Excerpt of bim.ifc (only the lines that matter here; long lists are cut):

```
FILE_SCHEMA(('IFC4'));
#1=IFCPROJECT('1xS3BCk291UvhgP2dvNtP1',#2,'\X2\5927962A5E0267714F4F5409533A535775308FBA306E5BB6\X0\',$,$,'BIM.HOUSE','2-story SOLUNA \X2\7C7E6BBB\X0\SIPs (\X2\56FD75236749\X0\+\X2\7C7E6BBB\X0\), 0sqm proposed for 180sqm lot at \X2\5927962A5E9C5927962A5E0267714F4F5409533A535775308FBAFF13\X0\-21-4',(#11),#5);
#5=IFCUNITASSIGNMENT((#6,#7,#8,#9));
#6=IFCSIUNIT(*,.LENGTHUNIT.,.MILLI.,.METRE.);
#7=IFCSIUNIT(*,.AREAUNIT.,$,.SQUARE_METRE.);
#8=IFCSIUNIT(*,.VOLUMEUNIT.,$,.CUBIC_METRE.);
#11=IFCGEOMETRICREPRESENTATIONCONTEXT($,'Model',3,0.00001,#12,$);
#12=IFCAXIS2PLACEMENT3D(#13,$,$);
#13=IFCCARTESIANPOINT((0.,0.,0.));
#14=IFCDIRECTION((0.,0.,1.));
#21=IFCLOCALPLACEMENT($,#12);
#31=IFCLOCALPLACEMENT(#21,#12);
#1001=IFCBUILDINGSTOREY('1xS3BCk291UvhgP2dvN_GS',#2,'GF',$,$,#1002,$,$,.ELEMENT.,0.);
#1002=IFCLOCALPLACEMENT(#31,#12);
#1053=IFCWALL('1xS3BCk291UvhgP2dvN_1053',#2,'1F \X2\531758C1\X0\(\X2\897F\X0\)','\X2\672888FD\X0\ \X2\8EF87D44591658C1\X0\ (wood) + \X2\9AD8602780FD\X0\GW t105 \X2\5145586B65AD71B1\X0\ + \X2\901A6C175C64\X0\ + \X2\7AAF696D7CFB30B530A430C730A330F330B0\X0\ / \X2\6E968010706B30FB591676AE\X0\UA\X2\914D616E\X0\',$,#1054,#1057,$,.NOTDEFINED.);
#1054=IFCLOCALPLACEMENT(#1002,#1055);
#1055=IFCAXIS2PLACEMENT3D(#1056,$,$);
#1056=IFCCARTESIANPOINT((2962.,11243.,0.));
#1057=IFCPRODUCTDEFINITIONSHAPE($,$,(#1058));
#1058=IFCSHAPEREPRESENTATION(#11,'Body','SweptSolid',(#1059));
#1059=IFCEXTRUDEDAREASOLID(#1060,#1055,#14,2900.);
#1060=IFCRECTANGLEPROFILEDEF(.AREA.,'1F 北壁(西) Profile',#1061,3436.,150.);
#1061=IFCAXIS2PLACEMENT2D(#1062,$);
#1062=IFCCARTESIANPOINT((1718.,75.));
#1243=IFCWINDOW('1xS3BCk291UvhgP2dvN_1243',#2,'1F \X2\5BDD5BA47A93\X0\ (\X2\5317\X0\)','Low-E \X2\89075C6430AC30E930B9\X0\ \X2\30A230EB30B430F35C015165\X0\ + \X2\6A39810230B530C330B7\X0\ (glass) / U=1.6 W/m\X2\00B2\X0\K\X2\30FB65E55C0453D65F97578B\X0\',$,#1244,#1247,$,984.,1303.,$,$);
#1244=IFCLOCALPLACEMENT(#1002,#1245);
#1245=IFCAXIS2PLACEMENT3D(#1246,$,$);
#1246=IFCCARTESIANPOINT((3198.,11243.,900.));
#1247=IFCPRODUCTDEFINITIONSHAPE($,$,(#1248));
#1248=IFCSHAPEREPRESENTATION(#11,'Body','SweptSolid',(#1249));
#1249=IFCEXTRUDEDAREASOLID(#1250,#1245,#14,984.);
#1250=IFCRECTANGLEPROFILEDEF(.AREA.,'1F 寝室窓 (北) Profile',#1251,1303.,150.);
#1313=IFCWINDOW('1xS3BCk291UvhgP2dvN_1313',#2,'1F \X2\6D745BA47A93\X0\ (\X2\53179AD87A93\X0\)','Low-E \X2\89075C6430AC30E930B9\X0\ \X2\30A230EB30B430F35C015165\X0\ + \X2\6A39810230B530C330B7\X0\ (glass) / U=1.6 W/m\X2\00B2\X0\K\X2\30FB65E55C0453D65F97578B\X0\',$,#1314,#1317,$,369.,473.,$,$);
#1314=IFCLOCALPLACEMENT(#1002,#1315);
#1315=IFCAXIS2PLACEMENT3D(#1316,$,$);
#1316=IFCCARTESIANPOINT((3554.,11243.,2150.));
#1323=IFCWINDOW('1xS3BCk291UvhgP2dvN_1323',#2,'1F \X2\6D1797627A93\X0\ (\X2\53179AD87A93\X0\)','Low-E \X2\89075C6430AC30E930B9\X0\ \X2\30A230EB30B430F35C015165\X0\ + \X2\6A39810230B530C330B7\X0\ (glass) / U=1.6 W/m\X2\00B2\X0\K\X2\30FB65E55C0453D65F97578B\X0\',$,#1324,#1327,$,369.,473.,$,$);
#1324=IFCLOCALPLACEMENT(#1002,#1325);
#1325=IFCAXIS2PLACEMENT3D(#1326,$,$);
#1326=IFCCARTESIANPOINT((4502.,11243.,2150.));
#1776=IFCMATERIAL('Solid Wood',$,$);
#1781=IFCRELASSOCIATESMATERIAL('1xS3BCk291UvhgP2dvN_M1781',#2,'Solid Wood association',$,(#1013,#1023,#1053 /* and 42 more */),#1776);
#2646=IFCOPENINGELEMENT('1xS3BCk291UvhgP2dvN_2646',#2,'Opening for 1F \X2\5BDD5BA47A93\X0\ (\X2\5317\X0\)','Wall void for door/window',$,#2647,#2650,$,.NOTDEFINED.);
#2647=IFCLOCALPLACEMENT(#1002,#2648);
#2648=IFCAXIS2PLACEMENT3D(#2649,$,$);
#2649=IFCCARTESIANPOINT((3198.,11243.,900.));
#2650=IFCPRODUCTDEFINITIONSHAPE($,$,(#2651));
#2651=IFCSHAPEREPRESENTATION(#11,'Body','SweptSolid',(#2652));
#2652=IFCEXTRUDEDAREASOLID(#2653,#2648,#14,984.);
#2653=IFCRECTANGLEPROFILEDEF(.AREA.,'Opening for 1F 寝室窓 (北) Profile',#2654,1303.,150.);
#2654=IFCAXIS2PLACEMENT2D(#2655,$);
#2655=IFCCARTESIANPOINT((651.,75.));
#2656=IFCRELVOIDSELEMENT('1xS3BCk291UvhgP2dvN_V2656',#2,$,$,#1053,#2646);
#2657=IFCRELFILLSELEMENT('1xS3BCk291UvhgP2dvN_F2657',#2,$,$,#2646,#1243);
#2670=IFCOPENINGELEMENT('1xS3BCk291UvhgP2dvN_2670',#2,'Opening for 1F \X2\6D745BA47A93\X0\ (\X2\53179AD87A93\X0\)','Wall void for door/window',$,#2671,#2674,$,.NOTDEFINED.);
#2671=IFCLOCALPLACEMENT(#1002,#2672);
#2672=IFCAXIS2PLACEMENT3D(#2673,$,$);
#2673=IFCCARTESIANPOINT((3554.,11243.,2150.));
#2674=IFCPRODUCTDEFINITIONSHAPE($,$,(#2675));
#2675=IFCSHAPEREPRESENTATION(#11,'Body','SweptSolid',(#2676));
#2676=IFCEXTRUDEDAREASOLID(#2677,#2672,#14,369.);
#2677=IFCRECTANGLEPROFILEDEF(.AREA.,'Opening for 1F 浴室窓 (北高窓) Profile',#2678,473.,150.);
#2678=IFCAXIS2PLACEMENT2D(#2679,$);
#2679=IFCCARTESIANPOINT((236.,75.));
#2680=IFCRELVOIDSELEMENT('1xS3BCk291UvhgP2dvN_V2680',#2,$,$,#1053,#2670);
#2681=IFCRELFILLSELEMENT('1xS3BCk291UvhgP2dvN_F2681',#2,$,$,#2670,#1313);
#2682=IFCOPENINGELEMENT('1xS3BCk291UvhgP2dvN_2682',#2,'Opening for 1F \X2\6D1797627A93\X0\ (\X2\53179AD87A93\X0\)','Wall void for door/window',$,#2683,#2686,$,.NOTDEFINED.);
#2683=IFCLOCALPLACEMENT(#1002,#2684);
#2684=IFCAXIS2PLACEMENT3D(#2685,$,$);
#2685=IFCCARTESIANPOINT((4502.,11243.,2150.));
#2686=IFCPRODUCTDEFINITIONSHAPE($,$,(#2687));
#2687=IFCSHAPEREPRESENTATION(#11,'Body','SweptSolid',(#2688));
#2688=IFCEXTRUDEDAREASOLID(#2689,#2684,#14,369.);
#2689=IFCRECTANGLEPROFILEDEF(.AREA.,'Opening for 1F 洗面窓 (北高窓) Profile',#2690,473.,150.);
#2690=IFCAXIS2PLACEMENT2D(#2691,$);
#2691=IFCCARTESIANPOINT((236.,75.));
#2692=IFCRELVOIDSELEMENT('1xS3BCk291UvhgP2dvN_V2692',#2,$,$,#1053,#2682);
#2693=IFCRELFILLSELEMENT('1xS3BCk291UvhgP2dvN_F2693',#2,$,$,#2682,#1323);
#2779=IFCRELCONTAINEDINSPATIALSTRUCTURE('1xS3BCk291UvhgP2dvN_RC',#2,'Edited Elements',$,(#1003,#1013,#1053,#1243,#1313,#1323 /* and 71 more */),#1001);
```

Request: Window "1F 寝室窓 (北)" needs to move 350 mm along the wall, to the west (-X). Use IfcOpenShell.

```python
import ifcopenshell
import ifcopenshell.api.geometry
import ifcopenshell.util.placement

model = ifcopenshell.open("bim.ifc")

window = model.by_guid("1xS3BCk291UvhgP2dvN_1243")
opening = window.FillsVoids[0].RelatingOpeningElement
wall = opening.VoidsElements[0].RelatingBuildingElement

wall_matrix = ifcopenshell.util.placement.get_local_placement(wall.ObjectPlacement)
shift = wall_matrix[:3, 0] * -350.0
before = ifcopenshell.util.placement.get_local_placement(window.ObjectPlacement)[:3, 3].copy()

# The window is not placed relative to its opening, so move both.
for product in (opening, window):
    matrix = ifcopenshell.util.placement.get_local_placement(product.ObjectPlacement)
    matrix[:3, 3] += shift
    ifcopenshell.api.geometry.edit_object_placement(model, product=product, matrix=matrix, is_si=False)

after = ifcopenshell.util.placement.get_local_placement(window.ObjectPlacement)[:3, 3]
print("window moved by", (after - before).round(3) + 0.0)

model.write("bim_rev.ifc")
```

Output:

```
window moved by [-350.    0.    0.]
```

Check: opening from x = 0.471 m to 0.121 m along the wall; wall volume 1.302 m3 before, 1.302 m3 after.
